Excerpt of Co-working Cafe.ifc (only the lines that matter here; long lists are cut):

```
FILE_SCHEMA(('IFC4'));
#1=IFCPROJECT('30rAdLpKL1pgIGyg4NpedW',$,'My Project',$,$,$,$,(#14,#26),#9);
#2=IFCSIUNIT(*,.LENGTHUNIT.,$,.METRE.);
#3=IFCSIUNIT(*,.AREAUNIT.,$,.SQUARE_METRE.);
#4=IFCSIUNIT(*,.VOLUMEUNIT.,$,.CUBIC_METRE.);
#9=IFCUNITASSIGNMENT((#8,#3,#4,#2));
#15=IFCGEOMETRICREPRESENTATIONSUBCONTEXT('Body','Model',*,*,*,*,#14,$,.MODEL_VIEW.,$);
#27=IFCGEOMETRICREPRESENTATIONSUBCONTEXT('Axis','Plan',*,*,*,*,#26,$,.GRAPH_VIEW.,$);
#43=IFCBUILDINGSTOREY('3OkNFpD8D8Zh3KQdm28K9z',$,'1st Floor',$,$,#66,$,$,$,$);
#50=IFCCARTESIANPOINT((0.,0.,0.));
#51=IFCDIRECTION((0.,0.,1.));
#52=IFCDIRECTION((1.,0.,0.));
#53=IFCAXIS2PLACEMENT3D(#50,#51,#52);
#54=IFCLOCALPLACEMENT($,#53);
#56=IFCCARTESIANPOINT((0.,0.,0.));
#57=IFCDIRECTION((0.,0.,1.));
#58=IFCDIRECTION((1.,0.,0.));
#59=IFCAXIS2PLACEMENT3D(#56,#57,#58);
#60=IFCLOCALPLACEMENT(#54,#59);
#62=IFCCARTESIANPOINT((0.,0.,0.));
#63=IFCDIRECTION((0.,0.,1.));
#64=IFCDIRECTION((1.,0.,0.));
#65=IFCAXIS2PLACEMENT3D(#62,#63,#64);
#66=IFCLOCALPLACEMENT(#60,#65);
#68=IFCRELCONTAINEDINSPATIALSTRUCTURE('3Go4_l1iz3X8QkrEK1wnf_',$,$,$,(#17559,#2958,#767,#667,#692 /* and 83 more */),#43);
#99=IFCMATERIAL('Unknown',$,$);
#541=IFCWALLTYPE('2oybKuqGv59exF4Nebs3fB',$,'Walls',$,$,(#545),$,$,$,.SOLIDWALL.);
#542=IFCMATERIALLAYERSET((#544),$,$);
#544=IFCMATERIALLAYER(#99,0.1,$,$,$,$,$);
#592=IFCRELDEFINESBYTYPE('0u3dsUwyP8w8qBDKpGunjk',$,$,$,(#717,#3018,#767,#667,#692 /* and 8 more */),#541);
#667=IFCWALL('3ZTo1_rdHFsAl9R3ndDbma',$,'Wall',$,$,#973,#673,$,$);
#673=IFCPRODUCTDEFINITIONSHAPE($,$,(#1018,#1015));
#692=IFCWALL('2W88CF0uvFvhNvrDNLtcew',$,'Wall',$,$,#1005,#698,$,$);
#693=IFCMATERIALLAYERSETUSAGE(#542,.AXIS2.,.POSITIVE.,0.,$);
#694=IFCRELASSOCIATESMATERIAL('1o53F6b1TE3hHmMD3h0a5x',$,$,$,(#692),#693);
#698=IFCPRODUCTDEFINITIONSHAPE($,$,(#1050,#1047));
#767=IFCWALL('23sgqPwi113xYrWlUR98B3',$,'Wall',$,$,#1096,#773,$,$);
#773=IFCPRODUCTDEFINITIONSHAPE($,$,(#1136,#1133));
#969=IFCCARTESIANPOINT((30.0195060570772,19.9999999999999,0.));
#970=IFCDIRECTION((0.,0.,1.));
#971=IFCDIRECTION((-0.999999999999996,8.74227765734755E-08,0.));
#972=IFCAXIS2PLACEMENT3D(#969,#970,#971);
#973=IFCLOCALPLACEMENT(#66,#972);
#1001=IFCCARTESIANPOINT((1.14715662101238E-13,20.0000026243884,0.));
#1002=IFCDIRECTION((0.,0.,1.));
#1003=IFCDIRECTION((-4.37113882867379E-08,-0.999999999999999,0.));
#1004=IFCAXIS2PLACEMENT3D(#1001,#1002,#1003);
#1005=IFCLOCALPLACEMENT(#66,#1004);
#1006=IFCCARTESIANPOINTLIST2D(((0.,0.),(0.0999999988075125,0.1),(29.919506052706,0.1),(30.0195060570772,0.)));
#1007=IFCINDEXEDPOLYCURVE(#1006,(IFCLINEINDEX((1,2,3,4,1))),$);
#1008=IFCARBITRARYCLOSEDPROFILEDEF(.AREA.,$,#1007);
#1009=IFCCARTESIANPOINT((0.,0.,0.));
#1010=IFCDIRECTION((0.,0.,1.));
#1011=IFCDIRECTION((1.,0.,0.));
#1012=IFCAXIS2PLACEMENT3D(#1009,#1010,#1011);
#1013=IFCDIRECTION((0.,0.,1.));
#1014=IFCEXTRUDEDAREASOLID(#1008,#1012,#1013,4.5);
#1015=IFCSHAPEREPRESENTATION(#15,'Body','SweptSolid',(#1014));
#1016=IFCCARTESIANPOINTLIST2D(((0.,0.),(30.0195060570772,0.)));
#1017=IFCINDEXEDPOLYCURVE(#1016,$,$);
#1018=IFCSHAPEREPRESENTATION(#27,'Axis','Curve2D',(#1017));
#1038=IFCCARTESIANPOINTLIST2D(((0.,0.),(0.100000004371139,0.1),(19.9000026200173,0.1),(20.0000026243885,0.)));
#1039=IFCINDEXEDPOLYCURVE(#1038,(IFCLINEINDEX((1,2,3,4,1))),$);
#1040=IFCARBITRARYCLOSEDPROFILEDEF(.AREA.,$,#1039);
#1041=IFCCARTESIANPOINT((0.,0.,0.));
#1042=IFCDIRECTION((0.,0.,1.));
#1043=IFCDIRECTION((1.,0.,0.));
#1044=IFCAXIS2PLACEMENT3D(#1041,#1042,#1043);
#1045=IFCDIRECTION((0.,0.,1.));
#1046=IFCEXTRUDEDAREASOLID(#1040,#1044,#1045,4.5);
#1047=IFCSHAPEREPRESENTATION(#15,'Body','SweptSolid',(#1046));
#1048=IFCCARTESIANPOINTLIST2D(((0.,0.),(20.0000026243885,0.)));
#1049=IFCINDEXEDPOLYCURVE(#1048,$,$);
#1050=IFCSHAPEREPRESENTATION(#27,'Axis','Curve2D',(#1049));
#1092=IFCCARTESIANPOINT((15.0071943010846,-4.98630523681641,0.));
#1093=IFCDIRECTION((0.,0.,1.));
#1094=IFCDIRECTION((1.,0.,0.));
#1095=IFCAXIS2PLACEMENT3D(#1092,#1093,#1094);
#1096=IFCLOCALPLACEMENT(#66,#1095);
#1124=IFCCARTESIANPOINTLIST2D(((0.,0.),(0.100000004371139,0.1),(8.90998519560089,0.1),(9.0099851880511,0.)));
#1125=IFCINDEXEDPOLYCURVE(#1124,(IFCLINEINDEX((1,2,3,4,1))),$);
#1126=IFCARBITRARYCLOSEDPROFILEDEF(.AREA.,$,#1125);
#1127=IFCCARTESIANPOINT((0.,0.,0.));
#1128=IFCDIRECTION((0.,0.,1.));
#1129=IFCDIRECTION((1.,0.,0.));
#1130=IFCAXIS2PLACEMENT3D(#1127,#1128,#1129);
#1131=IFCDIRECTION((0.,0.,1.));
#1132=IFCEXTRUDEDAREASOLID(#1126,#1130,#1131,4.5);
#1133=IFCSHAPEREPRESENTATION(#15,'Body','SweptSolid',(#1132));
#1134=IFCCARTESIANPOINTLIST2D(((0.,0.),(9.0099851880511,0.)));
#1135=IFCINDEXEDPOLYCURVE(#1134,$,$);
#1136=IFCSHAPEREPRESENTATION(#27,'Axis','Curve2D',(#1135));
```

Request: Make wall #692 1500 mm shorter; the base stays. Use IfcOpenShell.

```python
import ifcopenshell
import ifcopenshell.geom
import ifcopenshell.util.representation
import ifcopenshell.util.shape
import ifcopenshell.util.unit

model = ifcopenshell.open("Co-working Cafe.ifc")
unit_scale = ifcopenshell.util.unit.calculate_unit_scale(model)
settings = ifcopenshell.geom.settings()


def volume(element):
    """Net volume in cubic metres, openings subtracted."""
    shape = ifcopenshell.geom.create_shape(settings, element)
    return ifcopenshell.util.shape.get_volume(shape.geometry)


wall = model.by_guid("2W88CF0uvFvhNvrDNLtcew")
before = volume(wall)

body = ifcopenshell.util.representation.get_representation(wall, "Model", "Body")
solid = body.Items[0]
old_height = solid.Depth
solid.Depth -= 1.5 / unit_scale
after = volume(wall)

print(f"height {old_height:g} -> {solid.Depth:g}, volume {before:.3f} -> {after:.3f} m3")

model.write("Co-working Cafe_updated.ifc")
```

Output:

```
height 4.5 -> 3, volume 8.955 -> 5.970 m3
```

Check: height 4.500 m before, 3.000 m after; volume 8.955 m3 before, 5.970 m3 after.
